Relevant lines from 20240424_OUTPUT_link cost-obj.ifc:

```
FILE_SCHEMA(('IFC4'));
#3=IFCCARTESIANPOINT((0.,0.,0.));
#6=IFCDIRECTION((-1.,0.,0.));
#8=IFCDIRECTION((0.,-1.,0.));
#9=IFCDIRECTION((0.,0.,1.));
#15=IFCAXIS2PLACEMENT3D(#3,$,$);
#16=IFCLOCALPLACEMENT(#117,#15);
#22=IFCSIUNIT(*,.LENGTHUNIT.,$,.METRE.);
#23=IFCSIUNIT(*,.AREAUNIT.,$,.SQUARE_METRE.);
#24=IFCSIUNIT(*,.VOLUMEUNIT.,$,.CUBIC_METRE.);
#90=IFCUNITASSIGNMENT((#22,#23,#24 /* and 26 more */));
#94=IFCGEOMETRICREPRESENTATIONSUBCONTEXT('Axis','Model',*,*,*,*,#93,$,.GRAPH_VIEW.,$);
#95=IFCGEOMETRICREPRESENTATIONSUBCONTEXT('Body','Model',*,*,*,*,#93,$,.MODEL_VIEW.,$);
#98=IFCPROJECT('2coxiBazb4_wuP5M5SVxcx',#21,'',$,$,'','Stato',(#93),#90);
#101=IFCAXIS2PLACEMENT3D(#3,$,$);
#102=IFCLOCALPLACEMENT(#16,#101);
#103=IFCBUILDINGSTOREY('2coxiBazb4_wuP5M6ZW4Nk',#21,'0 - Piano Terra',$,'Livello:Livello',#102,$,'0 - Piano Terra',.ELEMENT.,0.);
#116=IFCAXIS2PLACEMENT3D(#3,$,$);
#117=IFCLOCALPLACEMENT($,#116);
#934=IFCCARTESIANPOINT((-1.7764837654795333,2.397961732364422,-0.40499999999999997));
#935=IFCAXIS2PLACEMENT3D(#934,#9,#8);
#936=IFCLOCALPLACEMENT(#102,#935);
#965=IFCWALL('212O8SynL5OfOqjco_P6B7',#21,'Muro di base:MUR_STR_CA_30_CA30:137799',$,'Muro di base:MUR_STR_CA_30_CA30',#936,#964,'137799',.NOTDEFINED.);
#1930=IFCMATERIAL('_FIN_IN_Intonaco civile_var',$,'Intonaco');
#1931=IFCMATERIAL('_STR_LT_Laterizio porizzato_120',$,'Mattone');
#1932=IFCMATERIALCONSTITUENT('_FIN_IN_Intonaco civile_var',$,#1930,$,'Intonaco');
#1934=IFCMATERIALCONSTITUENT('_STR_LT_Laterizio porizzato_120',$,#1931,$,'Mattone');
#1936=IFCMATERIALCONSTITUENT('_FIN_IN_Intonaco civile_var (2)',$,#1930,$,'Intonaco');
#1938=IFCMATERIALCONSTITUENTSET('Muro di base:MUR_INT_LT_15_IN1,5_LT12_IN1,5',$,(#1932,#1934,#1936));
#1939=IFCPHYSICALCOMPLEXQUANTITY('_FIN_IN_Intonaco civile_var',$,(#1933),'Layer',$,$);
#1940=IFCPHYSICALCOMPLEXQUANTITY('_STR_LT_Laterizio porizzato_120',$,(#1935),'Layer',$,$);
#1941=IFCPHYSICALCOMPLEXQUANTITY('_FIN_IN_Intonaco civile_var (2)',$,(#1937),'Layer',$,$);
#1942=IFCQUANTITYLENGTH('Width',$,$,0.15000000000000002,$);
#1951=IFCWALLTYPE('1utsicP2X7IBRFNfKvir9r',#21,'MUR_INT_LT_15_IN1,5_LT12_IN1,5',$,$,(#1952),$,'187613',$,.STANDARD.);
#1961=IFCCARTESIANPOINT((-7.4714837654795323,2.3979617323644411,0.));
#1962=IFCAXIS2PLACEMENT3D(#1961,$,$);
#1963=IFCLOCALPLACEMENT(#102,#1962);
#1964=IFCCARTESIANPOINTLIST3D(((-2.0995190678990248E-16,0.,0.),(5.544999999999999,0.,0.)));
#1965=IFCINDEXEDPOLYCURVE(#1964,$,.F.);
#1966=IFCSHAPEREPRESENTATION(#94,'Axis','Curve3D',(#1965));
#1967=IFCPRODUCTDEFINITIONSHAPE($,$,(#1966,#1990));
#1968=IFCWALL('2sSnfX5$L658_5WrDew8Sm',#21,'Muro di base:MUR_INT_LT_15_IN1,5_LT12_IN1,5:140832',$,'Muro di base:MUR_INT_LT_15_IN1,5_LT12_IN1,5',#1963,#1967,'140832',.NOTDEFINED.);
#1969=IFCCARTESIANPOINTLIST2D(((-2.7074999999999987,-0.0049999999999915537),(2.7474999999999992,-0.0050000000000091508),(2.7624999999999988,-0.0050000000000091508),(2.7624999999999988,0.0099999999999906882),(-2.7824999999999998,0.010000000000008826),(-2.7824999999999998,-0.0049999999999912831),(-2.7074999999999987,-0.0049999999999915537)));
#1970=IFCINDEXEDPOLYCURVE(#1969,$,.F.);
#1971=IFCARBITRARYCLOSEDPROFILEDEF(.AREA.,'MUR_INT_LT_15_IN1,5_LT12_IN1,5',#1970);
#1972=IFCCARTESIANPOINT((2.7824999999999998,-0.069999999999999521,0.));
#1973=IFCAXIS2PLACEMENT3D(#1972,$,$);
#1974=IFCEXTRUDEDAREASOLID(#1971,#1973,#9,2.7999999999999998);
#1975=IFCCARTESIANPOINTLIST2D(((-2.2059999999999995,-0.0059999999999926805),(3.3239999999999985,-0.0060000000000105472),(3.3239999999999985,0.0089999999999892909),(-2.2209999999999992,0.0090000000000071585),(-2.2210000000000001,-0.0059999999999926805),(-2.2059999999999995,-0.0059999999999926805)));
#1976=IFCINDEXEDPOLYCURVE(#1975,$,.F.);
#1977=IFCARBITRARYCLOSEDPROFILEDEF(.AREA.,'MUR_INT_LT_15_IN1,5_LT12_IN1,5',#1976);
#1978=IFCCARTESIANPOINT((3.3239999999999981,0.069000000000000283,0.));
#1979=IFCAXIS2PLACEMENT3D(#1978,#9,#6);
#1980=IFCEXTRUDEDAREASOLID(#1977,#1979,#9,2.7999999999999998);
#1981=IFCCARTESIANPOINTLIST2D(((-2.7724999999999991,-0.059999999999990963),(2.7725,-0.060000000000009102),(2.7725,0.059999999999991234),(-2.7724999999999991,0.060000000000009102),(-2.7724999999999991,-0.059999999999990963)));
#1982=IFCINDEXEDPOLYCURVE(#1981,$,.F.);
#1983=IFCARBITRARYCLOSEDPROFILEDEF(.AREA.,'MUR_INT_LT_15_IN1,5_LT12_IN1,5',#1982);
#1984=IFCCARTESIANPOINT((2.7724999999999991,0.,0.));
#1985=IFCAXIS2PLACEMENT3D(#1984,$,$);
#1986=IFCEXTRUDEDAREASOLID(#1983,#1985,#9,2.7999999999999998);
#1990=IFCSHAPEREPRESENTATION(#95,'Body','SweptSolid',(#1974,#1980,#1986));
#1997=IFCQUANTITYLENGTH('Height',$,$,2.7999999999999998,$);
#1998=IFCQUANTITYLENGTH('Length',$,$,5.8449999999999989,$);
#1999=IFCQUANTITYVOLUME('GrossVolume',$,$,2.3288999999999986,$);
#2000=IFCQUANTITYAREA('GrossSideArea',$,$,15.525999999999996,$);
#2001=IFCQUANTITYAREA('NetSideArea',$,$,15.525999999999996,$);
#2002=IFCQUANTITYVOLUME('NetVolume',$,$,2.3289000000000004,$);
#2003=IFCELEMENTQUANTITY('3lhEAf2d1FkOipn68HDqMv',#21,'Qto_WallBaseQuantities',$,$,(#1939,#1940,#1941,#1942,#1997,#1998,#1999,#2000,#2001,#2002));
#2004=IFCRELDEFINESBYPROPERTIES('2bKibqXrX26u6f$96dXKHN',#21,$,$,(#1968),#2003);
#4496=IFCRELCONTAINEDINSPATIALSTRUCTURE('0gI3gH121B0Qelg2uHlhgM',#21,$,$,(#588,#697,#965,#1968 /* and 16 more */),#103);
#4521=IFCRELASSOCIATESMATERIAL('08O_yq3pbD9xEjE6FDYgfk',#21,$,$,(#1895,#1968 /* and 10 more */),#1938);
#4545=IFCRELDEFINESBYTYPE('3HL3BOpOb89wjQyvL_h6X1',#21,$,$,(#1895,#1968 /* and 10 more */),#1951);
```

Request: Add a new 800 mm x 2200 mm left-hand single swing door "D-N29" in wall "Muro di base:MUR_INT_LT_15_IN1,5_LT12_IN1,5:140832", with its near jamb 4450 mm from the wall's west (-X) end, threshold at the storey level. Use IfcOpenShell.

```python
import numpy as np
import ifcopenshell
import ifcopenshell.api.feature
import ifcopenshell.api.geometry
import ifcopenshell.api.pset
import ifcopenshell.api.root
import ifcopenshell.api.spatial
import ifcopenshell.geom
import ifcopenshell.util.element
import ifcopenshell.util.placement
import ifcopenshell.util.representation
import ifcopenshell.util.shape
import ifcopenshell.util.unit

model = ifcopenshell.open("20240424_OUTPUT_link cost-obj.ifc")
unit_scale = ifcopenshell.util.unit.calculate_unit_scale(model)
area_scale = ifcopenshell.util.unit.calculate_unit_scale(model, "AREAUNIT")
volume_scale = ifcopenshell.util.unit.calculate_unit_scale(model, "VOLUMEUNIT")
settings = ifcopenshell.geom.settings()


def volume(element):
    """Net volume in cubic metres, openings subtracted."""
    shape = ifcopenshell.geom.create_shape(settings, element)
    return ifcopenshell.util.shape.get_volume(shape.geometry)


wall = model.by_id(1968)
storey = ifcopenshell.util.element.get_container(wall, ifc_class="IfcBuildingStorey")
context = ifcopenshell.util.representation.get_context(model, "Model", "Body", "MODEL_VIEW")
before = volume(wall)

width, height, from_end, sill = 0.8, 2.2, 4.45, 0.0  # metres

# The wall runs along its own X axis, and the end named is its -X end.
wall_shape = ifcopenshell.geom.create_shape(settings, wall)
x, y, z = ifcopenshell.util.shape.get_vertices(wall_shape.geometry).T
start = x.min() + from_end
face, thickness = float(y.min()), float(y.max() - y.min())
wall_matrix = ifcopenshell.util.placement.get_local_placement(wall.ObjectPlacement)
level = ifcopenshell.util.placement.get_local_placement(storey.ObjectPlacement)[2, 3]


def in_wall(x, y):
    """Placement at x, y metres in the wall's axes, at sill height."""
    matrix = wall_matrix.copy()
    matrix[:, 3] = wall_matrix @ np.array([x / unit_scale, y / unit_scale, 0.0, 1.0])
    matrix[2, 3] = level + sill / unit_scale
    return matrix


# Opening: a box that overshoots both wall faces by 50 mm.
opening = ifcopenshell.api.root.create_entity(model, ifc_class="IfcOpeningElement", predefined_type="OPENING")
box = ifcopenshell.api.geometry.add_wall_representation(
    model, context=context, length=width, height=height, thickness=thickness + 0.1
)
ifcopenshell.api.geometry.assign_representation(model, product=opening, representation=box)
ifcopenshell.api.geometry.edit_object_placement(model, product=opening, matrix=in_wall(start, face - 0.05), is_si=False)
ifcopenshell.api.feature.add_feature(model, feature=opening, element=wall)

door = ifcopenshell.api.root.create_entity(model, ifc_class="IfcDoor", name="D-N29", predefined_type="DOOR")
door.OverallWidth, door.OverallHeight = width / unit_scale, height / unit_scale
door.OperationType = "SINGLE_SWING_LEFT"
body = ifcopenshell.api.geometry.add_door_representation(
    model,
    context=context,
    overall_width=door.OverallWidth,
    overall_height=door.OverallHeight,
    operation_type="SINGLE_SWING_LEFT",
    lining_properties={"LiningDepth": thickness / unit_scale, "ThresholdDepth": thickness / unit_scale},
)
ifcopenshell.api.geometry.assign_representation(model, product=door, representation=body)
ifcopenshell.api.spatial.assign_container(model, products=[door], relating_structure=storey)
ifcopenshell.api.feature.add_filling(model, opening=opening, element=door)

# The lining spans the wall, so the door starts at the wall face.
ifcopenshell.api.geometry.edit_object_placement(model, product=door, matrix=in_wall(start, face), is_si=False)

after = volume(wall)

# Update the wall's stored quantities.
qto = model.by_id(ifcopenshell.util.element.get_pset(wall, "Qto_WallBaseQuantities", should_inherit=False)["id"])
ifcopenshell.api.pset.edit_qto(model, qto=qto, properties={
    "NetSideArea": after / thickness / area_scale,
    "NetVolume": after / volume_scale,
})

print(f"wall volume {before:.3f} -> {after:.3f} m3")

model.write("20240424_OUTPUT_link cost-obj-out.ifc")
```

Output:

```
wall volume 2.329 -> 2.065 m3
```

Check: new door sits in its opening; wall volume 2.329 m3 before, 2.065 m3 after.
